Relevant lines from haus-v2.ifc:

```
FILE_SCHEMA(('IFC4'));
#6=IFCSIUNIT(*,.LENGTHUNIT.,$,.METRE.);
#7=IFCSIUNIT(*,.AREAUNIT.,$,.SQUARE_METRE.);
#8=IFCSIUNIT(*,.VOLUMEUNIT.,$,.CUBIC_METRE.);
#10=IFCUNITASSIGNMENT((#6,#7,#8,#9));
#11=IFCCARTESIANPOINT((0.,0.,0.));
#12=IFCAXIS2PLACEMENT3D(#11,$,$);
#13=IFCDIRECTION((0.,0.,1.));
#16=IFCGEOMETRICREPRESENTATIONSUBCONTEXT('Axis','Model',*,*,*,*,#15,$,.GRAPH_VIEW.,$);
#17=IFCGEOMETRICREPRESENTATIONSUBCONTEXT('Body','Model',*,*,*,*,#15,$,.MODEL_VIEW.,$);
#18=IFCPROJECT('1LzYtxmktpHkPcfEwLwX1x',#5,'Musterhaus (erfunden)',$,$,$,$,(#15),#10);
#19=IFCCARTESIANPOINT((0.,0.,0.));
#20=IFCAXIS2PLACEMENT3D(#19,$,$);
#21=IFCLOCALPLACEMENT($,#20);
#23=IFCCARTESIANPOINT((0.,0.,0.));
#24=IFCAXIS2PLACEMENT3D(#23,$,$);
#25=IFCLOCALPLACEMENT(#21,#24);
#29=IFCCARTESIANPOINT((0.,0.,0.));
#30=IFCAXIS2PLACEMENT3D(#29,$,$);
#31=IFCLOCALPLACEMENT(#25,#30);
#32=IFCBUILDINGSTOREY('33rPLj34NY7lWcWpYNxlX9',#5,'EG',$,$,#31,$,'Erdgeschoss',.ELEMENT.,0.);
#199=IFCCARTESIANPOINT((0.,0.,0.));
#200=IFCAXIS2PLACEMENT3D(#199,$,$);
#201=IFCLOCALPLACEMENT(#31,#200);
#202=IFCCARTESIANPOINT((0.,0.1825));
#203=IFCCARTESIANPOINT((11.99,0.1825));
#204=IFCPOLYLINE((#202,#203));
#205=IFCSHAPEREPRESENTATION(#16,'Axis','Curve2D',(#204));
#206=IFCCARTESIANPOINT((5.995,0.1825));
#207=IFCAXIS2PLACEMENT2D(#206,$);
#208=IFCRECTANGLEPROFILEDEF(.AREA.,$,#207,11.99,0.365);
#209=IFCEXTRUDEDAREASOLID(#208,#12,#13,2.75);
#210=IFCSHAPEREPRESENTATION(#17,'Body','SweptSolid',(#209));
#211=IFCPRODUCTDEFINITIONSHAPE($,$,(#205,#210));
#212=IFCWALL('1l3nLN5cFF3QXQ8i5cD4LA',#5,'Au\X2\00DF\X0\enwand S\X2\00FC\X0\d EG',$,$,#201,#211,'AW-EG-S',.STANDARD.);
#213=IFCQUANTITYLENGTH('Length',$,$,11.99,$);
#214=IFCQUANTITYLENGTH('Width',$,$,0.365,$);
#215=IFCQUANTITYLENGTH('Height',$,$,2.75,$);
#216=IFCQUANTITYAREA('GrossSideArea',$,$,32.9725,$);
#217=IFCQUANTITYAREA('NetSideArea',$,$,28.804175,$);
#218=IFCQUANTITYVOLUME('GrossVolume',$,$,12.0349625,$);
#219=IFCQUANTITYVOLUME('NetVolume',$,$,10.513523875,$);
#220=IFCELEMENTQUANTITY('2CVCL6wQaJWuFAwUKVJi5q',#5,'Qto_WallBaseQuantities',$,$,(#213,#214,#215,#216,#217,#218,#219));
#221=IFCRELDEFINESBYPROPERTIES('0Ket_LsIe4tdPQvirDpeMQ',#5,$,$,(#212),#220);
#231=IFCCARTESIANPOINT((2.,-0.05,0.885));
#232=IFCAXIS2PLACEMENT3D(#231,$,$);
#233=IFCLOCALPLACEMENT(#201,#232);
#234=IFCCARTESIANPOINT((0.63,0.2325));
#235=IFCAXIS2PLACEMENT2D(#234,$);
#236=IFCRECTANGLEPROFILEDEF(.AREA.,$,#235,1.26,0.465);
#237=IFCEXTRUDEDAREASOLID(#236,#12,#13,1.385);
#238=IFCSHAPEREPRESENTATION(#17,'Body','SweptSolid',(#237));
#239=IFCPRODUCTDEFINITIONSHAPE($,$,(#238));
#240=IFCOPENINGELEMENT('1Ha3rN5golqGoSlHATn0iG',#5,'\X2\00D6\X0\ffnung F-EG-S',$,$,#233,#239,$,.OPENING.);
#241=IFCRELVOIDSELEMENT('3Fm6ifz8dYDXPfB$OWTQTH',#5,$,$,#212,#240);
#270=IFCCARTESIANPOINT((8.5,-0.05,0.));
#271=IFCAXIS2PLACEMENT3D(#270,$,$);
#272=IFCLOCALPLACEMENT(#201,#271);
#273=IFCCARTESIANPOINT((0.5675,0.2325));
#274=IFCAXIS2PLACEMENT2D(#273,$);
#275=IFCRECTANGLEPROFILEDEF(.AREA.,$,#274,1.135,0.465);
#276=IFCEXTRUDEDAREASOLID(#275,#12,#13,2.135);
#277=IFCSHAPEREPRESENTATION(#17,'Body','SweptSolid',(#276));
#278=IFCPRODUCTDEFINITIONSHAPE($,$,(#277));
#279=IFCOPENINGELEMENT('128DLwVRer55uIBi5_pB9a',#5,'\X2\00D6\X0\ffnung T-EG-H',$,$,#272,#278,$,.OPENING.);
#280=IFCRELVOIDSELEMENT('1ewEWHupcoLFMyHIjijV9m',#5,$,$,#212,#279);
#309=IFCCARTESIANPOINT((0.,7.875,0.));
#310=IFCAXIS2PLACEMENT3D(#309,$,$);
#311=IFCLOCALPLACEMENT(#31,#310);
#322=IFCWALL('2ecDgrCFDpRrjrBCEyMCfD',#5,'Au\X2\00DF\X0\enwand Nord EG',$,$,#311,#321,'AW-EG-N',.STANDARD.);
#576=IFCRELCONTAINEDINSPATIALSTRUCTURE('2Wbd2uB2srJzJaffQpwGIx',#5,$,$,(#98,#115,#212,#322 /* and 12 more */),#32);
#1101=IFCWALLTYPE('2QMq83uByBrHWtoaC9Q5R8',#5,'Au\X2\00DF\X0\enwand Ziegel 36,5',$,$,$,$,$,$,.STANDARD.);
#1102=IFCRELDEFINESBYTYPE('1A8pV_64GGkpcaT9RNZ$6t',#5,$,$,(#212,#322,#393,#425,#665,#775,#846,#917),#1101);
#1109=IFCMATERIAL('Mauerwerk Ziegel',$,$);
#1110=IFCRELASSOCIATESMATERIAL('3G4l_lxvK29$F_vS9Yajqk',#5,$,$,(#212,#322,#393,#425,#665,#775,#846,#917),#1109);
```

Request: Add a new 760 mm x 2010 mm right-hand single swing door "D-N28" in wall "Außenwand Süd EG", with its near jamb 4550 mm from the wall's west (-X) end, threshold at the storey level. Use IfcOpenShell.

```python
import numpy as np
import ifcopenshell
import ifcopenshell.api.feature
import ifcopenshell.api.geometry
import ifcopenshell.api.pset
import ifcopenshell.api.root
import ifcopenshell.api.spatial
import ifcopenshell.geom
import ifcopenshell.util.element
import ifcopenshell.util.placement
import ifcopenshell.util.representation
import ifcopenshell.util.shape
import ifcopenshell.util.unit

model = ifcopenshell.open("haus-v2.ifc")
unit_scale = ifcopenshell.util.unit.calculate_unit_scale(model)
area_scale = ifcopenshell.util.unit.calculate_unit_scale(model, "AREAUNIT")
volume_scale = ifcopenshell.util.unit.calculate_unit_scale(model, "VOLUMEUNIT")
settings = ifcopenshell.geom.settings()


def volume(element):
    """Net volume in cubic metres, openings subtracted."""
    shape = ifcopenshell.geom.create_shape(settings, element)
    return ifcopenshell.util.shape.get_volume(shape.geometry)


wall = model.by_guid("1l3nLN5cFF3QXQ8i5cD4LA")
storey = ifcopenshell.util.element.get_container(wall, ifc_class="IfcBuildingStorey")
context = ifcopenshell.util.representation.get_context(model, "Model", "Body", "MODEL_VIEW")
before = volume(wall)

width, height, from_end, sill = 0.76, 2.01, 4.55, 0.0  # metres

# The wall runs along its own X axis, and the end named is its -X end.
wall_shape = ifcopenshell.geom.create_shape(settings, wall)
x, y, z = ifcopenshell.util.shape.get_vertices(wall_shape.geometry).T
start = x.min() + from_end
face, thickness = float(y.min()), float(y.max() - y.min())
wall_matrix = ifcopenshell.util.placement.get_local_placement(wall.ObjectPlacement)
level = ifcopenshell.util.placement.get_local_placement(storey.ObjectPlacement)[2, 3]


def in_wall(x, y):
    """Placement at x, y metres in the wall's axes, at sill height."""
    matrix = wall_matrix.copy()
    matrix[:, 3] = wall_matrix @ np.array([x / unit_scale, y / unit_scale, 0.0, 1.0])
    matrix[2, 3] = level + sill / unit_scale
    return matrix


# Opening: a box that overshoots both wall faces by 50 mm.
opening = ifcopenshell.api.root.create_entity(model, ifc_class="IfcOpeningElement", predefined_type="OPENING")
box = ifcopenshell.api.geometry.add_wall_representation(
    model, context=context, length=width, height=height, thickness=thickness + 0.1
)
ifcopenshell.api.geometry.assign_representation(model, product=opening, representation=box)
ifcopenshell.api.geometry.edit_object_placement(model, product=opening, matrix=in_wall(start, face - 0.05), is_si=False)
ifcopenshell.api.feature.add_feature(model, feature=opening, element=wall)

door = ifcopenshell.api.root.create_entity(model, ifc_class="IfcDoor", name="D-N28", predefined_type="DOOR")
door.OverallWidth, door.OverallHeight = width / unit_scale, height / unit_scale
door.OperationType = "SINGLE_SWING_RIGHT"
body = ifcopenshell.api.geometry.add_door_representation(
    model,
    context=context,
    overall_width=door.OverallWidth,
    overall_height=door.OverallHeight,
    operation_type="SINGLE_SWING_RIGHT",
    lining_properties={"LiningDepth": thickness / unit_scale, "ThresholdDepth": thickness / unit_scale},
)
ifcopenshell.api.geometry.assign_representation(model, product=door, representation=body)
ifcopenshell.api.spatial.assign_container(model, products=[door], relating_structure=storey)
ifcopenshell.api.feature.add_filling(model, opening=opening, element=door)

# The lining spans the wall, so the door starts at the wall face.
ifcopenshell.api.geometry.edit_object_placement(model, product=door, matrix=in_wall(start, face), is_si=False)

after = volume(wall)

# Update the wall's stored quantities.
qto = model.by_id(ifcopenshell.util.element.get_pset(wall, "Qto_WallBaseQuantities", should_inherit=False)["id"])
ifcopenshell.api.pset.edit_qto(model, qto=qto, properties={
    "NetSideArea": after / thickness / area_scale,
    "NetVolume": after / volume_scale,
})

print(f"wall volume {before:.3f} -> {after:.3f} m3")

model.write("haus-v2_rev.ifc")
```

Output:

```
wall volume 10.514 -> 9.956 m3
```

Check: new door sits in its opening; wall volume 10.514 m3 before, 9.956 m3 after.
